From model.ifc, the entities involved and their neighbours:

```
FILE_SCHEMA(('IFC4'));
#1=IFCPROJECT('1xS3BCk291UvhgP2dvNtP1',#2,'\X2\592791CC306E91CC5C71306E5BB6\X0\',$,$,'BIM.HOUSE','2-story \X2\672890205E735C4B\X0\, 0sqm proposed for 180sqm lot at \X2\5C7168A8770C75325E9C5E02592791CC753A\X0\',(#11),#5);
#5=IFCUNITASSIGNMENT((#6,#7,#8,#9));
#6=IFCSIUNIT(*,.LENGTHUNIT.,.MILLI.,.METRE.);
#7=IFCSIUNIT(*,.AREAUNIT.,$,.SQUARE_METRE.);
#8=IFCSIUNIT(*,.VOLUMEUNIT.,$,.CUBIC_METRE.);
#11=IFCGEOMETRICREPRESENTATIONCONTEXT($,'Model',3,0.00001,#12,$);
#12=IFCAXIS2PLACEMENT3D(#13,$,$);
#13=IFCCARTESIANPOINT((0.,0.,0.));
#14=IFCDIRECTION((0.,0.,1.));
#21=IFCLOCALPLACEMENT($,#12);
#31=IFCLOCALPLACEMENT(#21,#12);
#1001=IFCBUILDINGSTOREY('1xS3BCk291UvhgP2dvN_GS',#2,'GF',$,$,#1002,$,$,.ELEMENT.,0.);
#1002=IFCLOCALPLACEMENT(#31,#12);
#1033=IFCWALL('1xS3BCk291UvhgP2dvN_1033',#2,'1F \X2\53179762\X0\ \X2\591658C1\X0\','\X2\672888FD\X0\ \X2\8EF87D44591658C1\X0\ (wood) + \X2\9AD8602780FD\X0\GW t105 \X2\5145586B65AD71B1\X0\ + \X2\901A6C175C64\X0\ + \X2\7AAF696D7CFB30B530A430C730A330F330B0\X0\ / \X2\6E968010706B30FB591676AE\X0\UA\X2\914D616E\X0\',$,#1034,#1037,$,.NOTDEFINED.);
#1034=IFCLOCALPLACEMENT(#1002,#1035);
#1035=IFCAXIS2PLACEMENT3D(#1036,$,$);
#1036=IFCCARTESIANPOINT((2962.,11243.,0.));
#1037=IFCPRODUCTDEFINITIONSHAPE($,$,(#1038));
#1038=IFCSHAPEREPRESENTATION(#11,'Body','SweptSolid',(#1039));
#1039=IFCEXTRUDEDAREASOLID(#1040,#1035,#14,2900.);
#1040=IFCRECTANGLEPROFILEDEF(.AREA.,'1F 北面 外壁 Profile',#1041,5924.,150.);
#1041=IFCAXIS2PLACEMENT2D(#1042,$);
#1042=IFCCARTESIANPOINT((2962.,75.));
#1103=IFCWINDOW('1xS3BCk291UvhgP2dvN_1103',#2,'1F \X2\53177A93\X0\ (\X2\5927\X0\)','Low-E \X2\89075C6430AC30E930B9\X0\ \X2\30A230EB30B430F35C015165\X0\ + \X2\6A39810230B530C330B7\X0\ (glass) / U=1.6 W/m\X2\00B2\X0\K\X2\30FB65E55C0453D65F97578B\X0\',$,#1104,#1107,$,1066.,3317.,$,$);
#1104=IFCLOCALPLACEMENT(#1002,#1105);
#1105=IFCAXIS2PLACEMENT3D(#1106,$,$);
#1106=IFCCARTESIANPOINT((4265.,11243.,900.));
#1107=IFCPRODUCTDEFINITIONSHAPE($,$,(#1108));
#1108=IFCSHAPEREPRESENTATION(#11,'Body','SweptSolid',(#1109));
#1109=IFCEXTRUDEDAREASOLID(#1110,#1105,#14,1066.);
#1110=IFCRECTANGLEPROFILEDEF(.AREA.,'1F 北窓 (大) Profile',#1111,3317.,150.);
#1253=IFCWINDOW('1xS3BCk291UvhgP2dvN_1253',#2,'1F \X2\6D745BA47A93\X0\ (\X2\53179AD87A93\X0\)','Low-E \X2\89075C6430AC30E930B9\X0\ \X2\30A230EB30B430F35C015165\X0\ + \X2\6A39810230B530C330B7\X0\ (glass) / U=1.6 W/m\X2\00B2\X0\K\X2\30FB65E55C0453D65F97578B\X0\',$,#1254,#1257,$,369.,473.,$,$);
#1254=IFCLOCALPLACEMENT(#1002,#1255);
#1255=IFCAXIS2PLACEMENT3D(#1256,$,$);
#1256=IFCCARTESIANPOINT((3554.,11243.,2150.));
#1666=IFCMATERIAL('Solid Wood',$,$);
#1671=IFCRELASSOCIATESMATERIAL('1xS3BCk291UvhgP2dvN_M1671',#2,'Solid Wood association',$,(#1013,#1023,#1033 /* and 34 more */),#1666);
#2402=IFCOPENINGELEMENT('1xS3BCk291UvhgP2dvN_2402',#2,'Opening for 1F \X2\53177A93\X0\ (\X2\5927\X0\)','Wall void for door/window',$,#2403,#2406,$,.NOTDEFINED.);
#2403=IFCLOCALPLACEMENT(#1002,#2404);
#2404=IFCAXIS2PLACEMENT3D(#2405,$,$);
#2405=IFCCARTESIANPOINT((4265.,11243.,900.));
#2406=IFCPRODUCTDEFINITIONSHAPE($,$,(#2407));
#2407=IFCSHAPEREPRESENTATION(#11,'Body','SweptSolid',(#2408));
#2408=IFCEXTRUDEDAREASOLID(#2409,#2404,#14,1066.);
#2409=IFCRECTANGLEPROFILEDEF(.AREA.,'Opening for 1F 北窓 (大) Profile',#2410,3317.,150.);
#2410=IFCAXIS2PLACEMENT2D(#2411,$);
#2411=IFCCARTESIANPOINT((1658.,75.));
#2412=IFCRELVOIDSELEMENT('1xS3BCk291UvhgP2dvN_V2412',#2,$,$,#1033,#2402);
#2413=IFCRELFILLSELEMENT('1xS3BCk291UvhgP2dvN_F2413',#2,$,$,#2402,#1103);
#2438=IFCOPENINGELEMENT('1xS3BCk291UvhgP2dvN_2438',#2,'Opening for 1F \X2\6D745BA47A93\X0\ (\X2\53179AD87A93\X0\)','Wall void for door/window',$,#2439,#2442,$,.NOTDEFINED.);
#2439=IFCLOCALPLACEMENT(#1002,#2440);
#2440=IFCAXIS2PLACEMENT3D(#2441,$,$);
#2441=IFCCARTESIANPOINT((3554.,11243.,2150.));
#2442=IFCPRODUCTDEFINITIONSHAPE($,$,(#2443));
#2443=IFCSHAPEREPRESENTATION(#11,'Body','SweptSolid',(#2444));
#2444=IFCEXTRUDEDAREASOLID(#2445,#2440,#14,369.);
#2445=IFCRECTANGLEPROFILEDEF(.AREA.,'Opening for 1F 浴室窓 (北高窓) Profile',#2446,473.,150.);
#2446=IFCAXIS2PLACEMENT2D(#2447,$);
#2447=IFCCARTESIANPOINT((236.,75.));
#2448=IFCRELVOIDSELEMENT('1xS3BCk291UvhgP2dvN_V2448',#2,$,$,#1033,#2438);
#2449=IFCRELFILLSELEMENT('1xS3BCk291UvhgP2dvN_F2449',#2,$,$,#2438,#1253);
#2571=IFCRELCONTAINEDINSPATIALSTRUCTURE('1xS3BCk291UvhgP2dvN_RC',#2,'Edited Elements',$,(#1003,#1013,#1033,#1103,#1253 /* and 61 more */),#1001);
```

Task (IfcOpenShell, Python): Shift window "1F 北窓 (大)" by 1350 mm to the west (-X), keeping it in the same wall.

```python
import ifcopenshell
import ifcopenshell.api.geometry
import ifcopenshell.util.placement
import ifcopenshell.util.unit

model = ifcopenshell.open("model.ifc")
unit_scale = ifcopenshell.util.unit.calculate_unit_scale(model)

window = model.by_guid("1xS3BCk291UvhgP2dvN_1103")
opening = window.FillsVoids[0].RelatingOpeningElement
wall = opening.VoidsElements[0].RelatingBuildingElement

wall_matrix = ifcopenshell.util.placement.get_local_placement(wall.ObjectPlacement)
shift = wall_matrix[:3, 0] * -1.35 / unit_scale
before = ifcopenshell.util.placement.get_local_placement(window.ObjectPlacement)[:3, 3].copy()

# The window is not placed relative to its opening, so move both.
for product in (opening, window):
    matrix = ifcopenshell.util.placement.get_local_placement(product.ObjectPlacement)
    matrix[:3, 3] += shift
    ifcopenshell.api.geometry.edit_object_placement(model, product=product, matrix=matrix, is_si=False)

after = ifcopenshell.util.placement.get_local_placement(window.ObjectPlacement)[:3, 3]
print("window moved by", (after - before).round(3) + 0.0)

model.write("model_rev.ifc")
```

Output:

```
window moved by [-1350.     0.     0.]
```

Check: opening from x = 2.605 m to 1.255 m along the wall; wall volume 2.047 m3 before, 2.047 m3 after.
